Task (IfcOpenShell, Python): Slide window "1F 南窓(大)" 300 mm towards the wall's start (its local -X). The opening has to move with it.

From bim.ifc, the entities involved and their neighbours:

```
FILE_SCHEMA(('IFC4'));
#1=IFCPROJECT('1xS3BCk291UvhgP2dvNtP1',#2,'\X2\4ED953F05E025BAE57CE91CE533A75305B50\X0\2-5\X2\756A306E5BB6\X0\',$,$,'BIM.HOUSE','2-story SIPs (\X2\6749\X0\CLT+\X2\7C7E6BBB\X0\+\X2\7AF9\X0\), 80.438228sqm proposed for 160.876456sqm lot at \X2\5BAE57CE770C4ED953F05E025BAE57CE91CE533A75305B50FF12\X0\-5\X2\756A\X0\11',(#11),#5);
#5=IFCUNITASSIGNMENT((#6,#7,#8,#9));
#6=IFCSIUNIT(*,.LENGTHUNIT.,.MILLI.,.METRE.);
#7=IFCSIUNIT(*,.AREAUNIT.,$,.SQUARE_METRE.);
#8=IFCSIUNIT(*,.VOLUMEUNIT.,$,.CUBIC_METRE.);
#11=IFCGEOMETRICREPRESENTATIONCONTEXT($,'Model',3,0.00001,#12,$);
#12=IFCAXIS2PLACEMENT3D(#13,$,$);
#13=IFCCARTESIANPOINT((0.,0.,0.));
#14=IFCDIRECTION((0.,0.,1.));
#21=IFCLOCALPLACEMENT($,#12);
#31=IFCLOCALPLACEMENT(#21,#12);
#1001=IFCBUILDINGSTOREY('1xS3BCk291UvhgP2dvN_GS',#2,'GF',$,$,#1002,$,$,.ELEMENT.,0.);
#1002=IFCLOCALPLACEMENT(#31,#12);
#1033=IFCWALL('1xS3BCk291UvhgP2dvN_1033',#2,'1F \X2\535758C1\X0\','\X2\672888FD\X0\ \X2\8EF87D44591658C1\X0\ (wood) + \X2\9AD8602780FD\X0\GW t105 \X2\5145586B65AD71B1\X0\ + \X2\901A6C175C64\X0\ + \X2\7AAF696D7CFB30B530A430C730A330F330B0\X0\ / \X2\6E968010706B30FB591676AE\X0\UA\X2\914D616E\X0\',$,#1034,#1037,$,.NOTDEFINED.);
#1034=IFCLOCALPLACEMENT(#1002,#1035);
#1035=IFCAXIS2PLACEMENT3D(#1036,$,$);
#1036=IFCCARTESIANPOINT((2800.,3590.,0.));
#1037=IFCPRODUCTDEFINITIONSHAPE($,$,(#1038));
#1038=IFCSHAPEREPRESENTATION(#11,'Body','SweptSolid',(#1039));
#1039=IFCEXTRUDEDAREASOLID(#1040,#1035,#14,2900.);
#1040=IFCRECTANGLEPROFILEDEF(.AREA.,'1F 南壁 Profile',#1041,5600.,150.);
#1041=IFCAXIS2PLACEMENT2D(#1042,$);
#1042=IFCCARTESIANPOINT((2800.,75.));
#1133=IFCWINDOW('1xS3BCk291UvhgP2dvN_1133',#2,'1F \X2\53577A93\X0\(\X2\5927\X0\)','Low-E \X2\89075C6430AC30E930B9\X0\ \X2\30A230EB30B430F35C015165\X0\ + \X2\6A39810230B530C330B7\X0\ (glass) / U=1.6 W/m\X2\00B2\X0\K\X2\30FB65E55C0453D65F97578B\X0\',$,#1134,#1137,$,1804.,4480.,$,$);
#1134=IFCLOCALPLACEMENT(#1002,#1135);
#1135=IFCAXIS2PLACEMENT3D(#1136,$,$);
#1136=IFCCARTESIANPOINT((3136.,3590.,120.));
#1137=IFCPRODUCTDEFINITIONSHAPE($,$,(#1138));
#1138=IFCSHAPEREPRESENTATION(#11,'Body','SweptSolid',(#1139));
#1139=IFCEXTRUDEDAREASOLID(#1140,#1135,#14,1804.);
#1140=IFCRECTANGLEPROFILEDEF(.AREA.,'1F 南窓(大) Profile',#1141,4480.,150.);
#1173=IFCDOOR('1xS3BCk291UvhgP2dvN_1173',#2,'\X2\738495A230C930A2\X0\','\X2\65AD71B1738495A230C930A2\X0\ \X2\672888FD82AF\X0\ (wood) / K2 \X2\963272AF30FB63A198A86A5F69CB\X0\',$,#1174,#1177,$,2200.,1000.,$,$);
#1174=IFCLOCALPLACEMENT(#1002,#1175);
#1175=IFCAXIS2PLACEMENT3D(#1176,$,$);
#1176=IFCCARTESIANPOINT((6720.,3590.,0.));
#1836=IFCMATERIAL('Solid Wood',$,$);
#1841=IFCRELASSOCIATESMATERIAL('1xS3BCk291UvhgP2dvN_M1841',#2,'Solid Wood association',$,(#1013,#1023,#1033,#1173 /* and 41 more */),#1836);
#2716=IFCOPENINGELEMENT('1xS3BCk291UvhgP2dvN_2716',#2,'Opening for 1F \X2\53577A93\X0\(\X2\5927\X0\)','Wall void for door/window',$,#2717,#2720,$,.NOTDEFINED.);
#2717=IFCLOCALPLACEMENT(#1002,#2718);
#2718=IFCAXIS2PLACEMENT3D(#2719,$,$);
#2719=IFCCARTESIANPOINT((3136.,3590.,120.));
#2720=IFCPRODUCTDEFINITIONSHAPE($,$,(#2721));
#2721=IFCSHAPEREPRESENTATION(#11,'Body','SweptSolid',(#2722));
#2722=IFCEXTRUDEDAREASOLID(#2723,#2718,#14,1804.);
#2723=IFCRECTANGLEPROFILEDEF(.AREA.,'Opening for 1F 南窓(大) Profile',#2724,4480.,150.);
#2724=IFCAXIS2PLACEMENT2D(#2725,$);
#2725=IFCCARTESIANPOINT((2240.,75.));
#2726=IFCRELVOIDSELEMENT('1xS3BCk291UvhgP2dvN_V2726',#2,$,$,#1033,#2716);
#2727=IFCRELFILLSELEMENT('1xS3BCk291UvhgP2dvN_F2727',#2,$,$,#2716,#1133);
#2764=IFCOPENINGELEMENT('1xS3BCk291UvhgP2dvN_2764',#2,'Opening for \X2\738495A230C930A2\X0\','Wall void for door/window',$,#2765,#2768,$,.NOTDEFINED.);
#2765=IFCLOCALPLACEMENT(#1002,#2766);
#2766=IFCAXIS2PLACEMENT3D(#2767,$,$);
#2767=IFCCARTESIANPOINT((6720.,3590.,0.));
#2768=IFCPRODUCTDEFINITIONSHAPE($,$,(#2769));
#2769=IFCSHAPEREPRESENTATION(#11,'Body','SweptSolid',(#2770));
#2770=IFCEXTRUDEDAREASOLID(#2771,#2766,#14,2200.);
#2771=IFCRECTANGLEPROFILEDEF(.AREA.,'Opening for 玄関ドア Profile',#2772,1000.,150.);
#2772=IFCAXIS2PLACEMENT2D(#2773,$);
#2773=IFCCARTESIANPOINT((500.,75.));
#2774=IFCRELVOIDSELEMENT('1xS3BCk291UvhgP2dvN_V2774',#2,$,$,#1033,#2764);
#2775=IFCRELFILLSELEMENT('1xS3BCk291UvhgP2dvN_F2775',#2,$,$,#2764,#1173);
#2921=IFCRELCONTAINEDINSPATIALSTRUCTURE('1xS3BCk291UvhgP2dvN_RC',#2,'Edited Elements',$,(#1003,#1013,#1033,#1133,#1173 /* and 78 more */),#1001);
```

```python
import ifcopenshell
import ifcopenshell.api.geometry
import ifcopenshell.util.placement

model = ifcopenshell.open("bim.ifc")

window = model.by_guid("1xS3BCk291UvhgP2dvN_1133")
opening = window.FillsVoids[0].RelatingOpeningElement
wall = opening.VoidsElements[0].RelatingBuildingElement

wall_matrix = ifcopenshell.util.placement.get_local_placement(wall.ObjectPlacement)
shift = wall_matrix[:3, 0] * -300.0
before = ifcopenshell.util.placement.get_local_placement(window.ObjectPlacement)[:3, 3].copy()

# The window is not placed relative to its opening, so move both.
for product in (opening, window):
    matrix = ifcopenshell.util.placement.get_local_placement(product.ObjectPlacement)
    matrix[:3, 3] += shift
    ifcopenshell.api.geometry.edit_object_placement(model, product=product, matrix=matrix, is_si=False)

after = ifcopenshell.util.placement.get_local_placement(window.ObjectPlacement)[:3, 3]
print("window moved by", (after - before).round(3) + 0.0)

model.write("bim_updated.ifc")
```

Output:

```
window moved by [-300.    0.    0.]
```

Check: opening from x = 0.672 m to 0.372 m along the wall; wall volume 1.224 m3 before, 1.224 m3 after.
